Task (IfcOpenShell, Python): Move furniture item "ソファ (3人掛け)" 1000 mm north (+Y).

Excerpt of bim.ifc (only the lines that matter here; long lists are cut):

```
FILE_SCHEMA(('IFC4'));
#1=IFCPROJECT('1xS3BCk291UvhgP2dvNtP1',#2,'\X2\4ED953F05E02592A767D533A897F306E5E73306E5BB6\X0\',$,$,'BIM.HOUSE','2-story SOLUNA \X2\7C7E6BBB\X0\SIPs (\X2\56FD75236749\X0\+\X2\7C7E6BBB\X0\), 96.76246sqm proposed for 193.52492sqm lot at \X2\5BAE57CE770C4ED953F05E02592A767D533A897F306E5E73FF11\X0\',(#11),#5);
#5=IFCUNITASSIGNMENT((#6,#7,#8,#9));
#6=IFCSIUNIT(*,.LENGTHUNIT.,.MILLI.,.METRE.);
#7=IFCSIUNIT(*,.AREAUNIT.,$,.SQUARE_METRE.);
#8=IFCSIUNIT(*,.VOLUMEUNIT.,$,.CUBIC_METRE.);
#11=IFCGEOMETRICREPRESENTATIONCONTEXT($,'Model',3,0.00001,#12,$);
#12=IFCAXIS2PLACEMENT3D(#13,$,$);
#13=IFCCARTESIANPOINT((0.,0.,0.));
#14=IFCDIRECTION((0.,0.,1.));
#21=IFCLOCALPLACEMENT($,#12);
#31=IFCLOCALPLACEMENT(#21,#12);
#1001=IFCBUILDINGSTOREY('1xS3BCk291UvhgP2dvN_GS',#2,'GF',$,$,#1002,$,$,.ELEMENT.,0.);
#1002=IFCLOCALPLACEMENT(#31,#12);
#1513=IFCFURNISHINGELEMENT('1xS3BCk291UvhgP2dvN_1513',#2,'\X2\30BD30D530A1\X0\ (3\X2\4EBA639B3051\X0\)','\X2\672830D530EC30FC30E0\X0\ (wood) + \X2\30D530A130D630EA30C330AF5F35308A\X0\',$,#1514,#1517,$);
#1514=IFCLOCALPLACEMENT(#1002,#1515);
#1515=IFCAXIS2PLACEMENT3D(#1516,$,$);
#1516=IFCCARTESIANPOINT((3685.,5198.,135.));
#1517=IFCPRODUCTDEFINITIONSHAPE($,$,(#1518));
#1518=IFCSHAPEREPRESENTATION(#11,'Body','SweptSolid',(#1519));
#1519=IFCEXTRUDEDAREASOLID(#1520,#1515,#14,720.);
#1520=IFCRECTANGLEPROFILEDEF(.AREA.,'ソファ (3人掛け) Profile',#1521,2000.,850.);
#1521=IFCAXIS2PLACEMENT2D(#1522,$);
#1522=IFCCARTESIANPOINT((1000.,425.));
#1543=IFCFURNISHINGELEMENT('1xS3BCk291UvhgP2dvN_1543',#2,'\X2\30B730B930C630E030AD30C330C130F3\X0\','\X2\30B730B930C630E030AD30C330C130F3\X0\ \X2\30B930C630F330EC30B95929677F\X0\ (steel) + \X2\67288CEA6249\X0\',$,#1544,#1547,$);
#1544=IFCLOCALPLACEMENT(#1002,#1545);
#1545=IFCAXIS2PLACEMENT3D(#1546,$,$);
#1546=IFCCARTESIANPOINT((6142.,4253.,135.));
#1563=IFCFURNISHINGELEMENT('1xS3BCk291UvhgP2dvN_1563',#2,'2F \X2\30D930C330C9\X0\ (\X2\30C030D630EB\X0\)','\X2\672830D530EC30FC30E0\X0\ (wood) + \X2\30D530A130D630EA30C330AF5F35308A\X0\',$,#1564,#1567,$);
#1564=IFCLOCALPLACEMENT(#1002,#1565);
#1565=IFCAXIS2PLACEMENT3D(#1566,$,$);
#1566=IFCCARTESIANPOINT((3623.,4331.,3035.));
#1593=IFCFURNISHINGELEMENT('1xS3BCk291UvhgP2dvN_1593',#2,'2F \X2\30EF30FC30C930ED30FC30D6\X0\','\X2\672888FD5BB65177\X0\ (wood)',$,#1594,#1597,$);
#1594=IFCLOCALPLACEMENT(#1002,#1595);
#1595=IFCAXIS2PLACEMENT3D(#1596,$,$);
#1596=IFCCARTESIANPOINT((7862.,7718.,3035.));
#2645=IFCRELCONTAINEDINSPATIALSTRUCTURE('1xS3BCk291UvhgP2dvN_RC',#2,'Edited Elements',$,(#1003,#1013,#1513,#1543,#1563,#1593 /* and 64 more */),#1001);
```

```python
import ifcopenshell
import ifcopenshell.api.geometry
import ifcopenshell.util.placement
import ifcopenshell.util.unit

model = ifcopenshell.open("bim.ifc")
unit_scale = ifcopenshell.util.unit.calculate_unit_scale(model)

item = model.by_guid("1xS3BCk291UvhgP2dvN_1513")
matrix = ifcopenshell.util.placement.get_local_placement(item.ObjectPlacement)
matrix[1, 3] += 1 / unit_scale
ifcopenshell.api.geometry.edit_object_placement(model, product=item, matrix=matrix, is_si=False)

print(ifcopenshell.util.placement.get_local_placement(item.ObjectPlacement).round(3) + 0.0)

model.write("bim_v2.ifc")
```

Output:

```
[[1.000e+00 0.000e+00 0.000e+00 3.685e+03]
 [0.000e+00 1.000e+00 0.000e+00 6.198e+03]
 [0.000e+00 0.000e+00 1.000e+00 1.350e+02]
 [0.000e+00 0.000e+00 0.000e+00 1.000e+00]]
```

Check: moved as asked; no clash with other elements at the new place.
